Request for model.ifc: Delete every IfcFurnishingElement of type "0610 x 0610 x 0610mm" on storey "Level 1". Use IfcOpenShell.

First a look at what the model holds.

```python
import ifcopenshell
import ifcopenshell.util.element

model = ifcopenshell.open("model.ifc")
print(model.schema)
storey = next(s for s in model.by_type("IfcBuildingStorey") if s.Name == "Level 1")
furniture = [e for e in ifcopenshell.util.element.get_decomposition(storey) if e.is_a("IfcFurnishingElement")]
seen = {}
for e in furniture:
    element_type = ifcopenshell.util.element.get_type(e)
    name = element_type.Name if element_type not in (None, e) else None
    seen[name] = seen.get(name, 0) + 1
for name, count in sorted(seen.items(), key=str):
    print(count, "x", name)
```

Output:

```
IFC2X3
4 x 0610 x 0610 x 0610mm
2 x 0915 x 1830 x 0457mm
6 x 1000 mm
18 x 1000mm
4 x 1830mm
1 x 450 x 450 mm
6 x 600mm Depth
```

```python
import ifcopenshell
import ifcopenshell.api.root
import ifcopenshell.util.element

model = ifcopenshell.open("model.ifc")

storey = next(s for s in model.by_type("IfcBuildingStorey") if s.Name == "Level 1")
furniture = [e for e in ifcopenshell.util.element.get_decomposition(storey) if e.is_a("IfcFurnishingElement")]
targets = [e for e in furniture if (t := ifcopenshell.util.element.get_type(e)) not in (None, e) and t.Name == "0610 x 0610 x 0610mm"]

for e in targets:
    ifcopenshell.api.root.remove_product(model, product=e)
print(len(targets), "removed")

model.write("model-out.ifc")
```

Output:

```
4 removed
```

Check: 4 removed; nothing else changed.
